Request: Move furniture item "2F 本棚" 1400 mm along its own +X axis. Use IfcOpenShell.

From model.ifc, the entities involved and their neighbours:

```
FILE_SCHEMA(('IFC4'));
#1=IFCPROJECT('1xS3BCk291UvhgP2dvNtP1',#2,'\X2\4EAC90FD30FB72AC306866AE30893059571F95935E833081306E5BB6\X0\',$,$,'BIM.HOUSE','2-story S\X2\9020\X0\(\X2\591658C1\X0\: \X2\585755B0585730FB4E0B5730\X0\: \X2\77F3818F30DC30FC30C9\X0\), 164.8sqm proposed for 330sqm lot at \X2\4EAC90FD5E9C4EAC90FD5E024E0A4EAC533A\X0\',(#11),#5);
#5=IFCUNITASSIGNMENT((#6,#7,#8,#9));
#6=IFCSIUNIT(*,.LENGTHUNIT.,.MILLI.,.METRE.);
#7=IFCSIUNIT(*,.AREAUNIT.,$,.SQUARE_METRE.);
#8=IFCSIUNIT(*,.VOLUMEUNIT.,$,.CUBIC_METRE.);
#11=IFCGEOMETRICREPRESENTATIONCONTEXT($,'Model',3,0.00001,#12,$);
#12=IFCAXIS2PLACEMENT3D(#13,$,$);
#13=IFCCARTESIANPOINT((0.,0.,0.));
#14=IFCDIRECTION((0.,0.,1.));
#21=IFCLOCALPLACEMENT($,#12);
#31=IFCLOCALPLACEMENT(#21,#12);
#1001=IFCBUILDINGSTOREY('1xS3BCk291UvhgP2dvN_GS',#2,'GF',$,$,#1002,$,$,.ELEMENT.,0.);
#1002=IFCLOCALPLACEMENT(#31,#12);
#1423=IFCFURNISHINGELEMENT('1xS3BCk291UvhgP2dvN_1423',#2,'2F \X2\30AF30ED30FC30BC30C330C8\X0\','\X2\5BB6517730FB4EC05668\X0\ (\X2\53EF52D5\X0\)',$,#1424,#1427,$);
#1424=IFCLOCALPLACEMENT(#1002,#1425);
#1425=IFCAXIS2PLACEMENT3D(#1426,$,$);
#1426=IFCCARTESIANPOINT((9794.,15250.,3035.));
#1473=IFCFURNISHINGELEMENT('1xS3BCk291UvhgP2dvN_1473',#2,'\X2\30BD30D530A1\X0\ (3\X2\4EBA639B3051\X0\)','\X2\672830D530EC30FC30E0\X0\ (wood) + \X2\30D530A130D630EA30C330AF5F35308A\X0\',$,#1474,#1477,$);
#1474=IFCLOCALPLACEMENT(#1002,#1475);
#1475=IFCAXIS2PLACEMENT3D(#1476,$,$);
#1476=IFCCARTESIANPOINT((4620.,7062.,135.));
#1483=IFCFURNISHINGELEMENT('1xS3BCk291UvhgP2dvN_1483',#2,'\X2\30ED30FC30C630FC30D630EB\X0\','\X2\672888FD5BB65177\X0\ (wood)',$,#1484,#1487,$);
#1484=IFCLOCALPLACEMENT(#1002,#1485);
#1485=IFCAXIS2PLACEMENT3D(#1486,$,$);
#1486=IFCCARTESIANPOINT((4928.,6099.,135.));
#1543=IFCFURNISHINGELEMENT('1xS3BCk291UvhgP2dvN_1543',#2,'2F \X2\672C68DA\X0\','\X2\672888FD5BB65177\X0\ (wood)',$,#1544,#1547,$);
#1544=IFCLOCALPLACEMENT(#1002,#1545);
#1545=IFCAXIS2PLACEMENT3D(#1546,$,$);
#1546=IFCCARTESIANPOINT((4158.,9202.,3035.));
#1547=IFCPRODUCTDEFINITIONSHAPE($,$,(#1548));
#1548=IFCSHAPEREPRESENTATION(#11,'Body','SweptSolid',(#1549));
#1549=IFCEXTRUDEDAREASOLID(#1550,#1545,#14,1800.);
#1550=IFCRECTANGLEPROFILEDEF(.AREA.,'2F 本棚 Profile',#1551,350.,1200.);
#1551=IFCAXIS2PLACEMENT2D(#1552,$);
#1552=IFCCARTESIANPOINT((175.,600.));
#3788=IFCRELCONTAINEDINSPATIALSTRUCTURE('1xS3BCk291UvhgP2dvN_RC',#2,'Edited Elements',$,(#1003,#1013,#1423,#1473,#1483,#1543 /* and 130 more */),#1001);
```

```python
import ifcopenshell
import ifcopenshell.api.geometry
import ifcopenshell.util.placement

model = ifcopenshell.open("model.ifc")

item = model.by_guid("1xS3BCk291UvhgP2dvN_1543")
matrix = ifcopenshell.util.placement.get_local_placement(item.ObjectPlacement)
matrix[:3, 3] += matrix[:3, 0] * 1400.0
ifcopenshell.api.geometry.edit_object_placement(model, product=item, matrix=matrix, is_si=False)

print(ifcopenshell.util.placement.get_local_placement(item.ObjectPlacement).round(3) + 0.0)

model.write("model_v2.ifc")
```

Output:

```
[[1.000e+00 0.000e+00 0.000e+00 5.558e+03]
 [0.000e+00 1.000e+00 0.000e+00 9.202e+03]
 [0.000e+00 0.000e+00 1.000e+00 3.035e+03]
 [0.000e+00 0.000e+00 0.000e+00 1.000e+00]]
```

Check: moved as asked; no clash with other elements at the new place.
